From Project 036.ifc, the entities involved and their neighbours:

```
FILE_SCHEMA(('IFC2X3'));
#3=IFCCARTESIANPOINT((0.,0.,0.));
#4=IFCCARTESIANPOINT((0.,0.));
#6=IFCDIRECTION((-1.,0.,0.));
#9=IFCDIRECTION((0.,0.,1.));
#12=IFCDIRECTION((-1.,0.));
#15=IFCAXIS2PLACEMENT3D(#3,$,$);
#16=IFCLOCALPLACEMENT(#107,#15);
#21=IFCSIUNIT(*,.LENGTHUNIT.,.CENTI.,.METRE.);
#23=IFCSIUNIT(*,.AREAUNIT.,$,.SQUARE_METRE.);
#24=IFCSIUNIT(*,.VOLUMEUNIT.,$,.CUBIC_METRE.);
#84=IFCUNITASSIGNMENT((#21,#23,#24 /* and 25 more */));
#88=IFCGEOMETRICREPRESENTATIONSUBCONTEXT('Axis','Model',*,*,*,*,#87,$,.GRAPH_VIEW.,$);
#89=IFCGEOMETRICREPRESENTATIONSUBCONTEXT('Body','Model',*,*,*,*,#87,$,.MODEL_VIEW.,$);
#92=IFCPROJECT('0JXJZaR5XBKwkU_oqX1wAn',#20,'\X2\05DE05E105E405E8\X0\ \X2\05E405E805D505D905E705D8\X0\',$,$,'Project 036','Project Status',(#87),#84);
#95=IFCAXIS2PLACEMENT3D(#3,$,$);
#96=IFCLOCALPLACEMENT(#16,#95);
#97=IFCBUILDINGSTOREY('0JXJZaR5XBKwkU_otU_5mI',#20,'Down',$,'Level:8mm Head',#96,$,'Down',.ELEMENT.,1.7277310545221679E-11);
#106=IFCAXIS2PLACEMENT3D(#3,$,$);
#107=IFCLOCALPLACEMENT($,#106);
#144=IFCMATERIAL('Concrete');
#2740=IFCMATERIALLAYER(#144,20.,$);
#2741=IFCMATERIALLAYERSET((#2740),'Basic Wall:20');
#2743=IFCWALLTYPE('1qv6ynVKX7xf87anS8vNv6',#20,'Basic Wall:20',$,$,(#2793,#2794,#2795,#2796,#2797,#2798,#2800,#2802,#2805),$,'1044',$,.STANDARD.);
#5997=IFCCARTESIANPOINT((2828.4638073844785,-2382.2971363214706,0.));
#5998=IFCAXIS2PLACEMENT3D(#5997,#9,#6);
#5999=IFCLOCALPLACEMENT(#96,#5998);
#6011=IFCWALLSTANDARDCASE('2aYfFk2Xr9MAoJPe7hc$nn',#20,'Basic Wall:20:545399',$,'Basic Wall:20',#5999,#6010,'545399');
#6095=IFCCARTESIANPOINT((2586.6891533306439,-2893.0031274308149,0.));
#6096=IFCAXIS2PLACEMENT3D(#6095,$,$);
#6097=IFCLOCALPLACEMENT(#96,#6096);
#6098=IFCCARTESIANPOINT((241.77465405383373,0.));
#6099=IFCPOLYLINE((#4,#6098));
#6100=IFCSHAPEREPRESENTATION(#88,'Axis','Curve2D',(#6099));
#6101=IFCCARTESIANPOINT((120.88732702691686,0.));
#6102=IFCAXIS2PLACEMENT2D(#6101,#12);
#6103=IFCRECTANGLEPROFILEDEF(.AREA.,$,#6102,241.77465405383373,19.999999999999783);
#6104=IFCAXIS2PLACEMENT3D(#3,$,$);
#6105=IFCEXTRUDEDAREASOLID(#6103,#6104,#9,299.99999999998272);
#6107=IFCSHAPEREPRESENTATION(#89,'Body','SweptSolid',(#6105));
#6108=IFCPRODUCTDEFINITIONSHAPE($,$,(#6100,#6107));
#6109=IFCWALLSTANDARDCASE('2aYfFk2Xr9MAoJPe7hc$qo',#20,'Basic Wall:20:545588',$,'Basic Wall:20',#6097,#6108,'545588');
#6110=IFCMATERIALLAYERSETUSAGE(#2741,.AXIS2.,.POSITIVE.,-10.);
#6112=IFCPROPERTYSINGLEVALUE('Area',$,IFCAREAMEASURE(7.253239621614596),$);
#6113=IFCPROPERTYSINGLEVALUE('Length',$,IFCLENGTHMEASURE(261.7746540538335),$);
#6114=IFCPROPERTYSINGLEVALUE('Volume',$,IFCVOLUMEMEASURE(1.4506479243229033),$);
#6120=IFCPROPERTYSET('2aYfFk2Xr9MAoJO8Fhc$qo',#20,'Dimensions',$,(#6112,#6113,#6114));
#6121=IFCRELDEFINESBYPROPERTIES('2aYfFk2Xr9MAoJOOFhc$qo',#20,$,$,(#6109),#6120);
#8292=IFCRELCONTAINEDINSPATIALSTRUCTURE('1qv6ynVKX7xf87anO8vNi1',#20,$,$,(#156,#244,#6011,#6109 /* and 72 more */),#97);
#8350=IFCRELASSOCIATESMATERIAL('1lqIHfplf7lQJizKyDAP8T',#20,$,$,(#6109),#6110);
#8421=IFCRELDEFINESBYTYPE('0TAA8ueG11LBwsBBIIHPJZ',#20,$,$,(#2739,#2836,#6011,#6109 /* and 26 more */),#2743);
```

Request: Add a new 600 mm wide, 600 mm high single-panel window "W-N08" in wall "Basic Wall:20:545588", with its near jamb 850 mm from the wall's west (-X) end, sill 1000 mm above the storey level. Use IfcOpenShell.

```python
import numpy as np
import ifcopenshell
import ifcopenshell.api.feature
import ifcopenshell.api.geometry
import ifcopenshell.api.pset
import ifcopenshell.api.root
import ifcopenshell.api.spatial
import ifcopenshell.api.type
import ifcopenshell.geom
import ifcopenshell.util.element
import ifcopenshell.util.placement
import ifcopenshell.util.representation
import ifcopenshell.util.shape
import ifcopenshell.util.unit

model = ifcopenshell.open("Project 036.ifc")
unit_scale = ifcopenshell.util.unit.calculate_unit_scale(model)
area_scale = ifcopenshell.util.unit.calculate_unit_scale(model, "AREAUNIT")
volume_scale = ifcopenshell.util.unit.calculate_unit_scale(model, "VOLUMEUNIT")
settings = ifcopenshell.geom.settings()


def volume(element):
    """Net volume in cubic metres, openings subtracted."""
    shape = ifcopenshell.geom.create_shape(settings, element)
    return ifcopenshell.util.shape.get_volume(shape.geometry)


wall = model.by_guid("2aYfFk2Xr9MAoJPe7hc$qo")
storey = ifcopenshell.util.element.get_container(wall, ifc_class="IfcBuildingStorey")
context = ifcopenshell.util.representation.get_context(model, "Model", "Body", "MODEL_VIEW")
before = volume(wall)

width, height, from_end, sill = 0.6, 0.6, 0.85, 1  # metres

# The wall runs along its own X axis, and the end named is its -X end.
wall_shape = ifcopenshell.geom.create_shape(settings, wall)
x, y, z = ifcopenshell.util.shape.get_vertices(wall_shape.geometry).T
start = x.min() + from_end
face, thickness = float(y.min()), float(y.max() - y.min())
wall_matrix = ifcopenshell.util.placement.get_local_placement(wall.ObjectPlacement)
level = ifcopenshell.util.placement.get_local_placement(storey.ObjectPlacement)[2, 3]


def in_wall(x, y):
    """Placement at x, y metres in the wall's axes, at sill height."""
    matrix = wall_matrix.copy()
    matrix[:, 3] = wall_matrix @ np.array([x / unit_scale, y / unit_scale, 0.0, 1.0])
    matrix[2, 3] = level + sill / unit_scale
    return matrix


# Opening: a box that overshoots both wall faces by 50 mm.
opening = ifcopenshell.api.root.create_entity(model, ifc_class="IfcOpeningElement")
box = ifcopenshell.api.geometry.add_wall_representation(
    model, context=context, length=width, height=height, thickness=thickness + 0.1
)
ifcopenshell.api.geometry.assign_representation(model, product=opening, representation=box)
ifcopenshell.api.geometry.edit_object_placement(model, product=opening, matrix=in_wall(start, face - 0.05), is_si=False)
ifcopenshell.api.feature.add_feature(model, feature=opening, element=wall)

window = ifcopenshell.api.root.create_entity(model, ifc_class="IfcWindow", name="W-N08")
window.OverallWidth, window.OverallHeight = width / unit_scale, height / unit_scale
body = ifcopenshell.api.geometry.add_window_representation(
    model,
    context=context,
    overall_width=window.OverallWidth,
    overall_height=window.OverallHeight,
    partition_type="SINGLE_PANEL",
)
ifcopenshell.api.geometry.assign_representation(model, product=window, representation=body)
ifcopenshell.api.spatial.assign_container(model, products=[window], relating_structure=storey)
fills = ifcopenshell.api.feature.add_filling(model, opening=opening, element=window)
fills.OwnerHistory = window.OwnerHistory  # required in IFC2X3

# IFC2X3 keeps the operation on the window style.
style = ifcopenshell.api.root.create_entity(model, ifc_class="IfcWindowStyle", name="W-N08")
style.OperationType, style.ConstructionType = "SINGLE_PANEL", "NOTDEFINED"
style.ParameterTakesPrecedence = style.Sizeable = False
ifcopenshell.api.type.assign_type(model, related_objects=[window], relating_type=style)

# Centre the window in the wall's thickness.
ifcopenshell.api.geometry.edit_object_placement(model, product=window, matrix=in_wall(start, face), is_si=False)
window_shape = ifcopenshell.geom.create_shape(settings, window)
depth = ifcopenshell.util.shape.get_vertices(window_shape.geometry)[:, 1]
offset = face + thickness / 2 - (depth.min() + depth.max()) / 2
ifcopenshell.api.geometry.edit_object_placement(model, product=window, matrix=in_wall(start, offset), is_si=False)

after = volume(wall)

# Update the wall's stored quantities.
pset = model.by_id(ifcopenshell.util.element.get_pset(wall, "Dimensions", should_inherit=False)["id"])
ifcopenshell.api.pset.edit_pset(model, pset=pset, properties={
    "Area": model.create_entity("IfcAreaMeasure", after / thickness / area_scale),
    "Volume": model.create_entity("IfcVolumeMeasure", after / volume_scale),
})

print(f"wall volume {before:.3f} -> {after:.3f} m3")

model.write("Project 036_updated.ifc")
```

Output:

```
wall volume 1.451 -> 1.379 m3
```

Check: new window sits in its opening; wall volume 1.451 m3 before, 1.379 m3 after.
